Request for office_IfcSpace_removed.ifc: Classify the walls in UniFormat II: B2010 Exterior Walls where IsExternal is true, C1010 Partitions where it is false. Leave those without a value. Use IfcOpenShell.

First a look at what the model holds.

```python
import ifcopenshell
import ifcopenshell.util.element

model = ifcopenshell.open("office_IfcSpace_removed.ifc")
print(model.schema)
print("classifications:", [c.Name for c in model.by_type("IfcClassification")])
values = [ifcopenshell.util.element.get_pset(e, "Pset_WallCommon", "IsExternal") for e in model.by_type("IfcWall")]
for value in (True, False, None):
    print("IsExternal", value, values.count(value))
```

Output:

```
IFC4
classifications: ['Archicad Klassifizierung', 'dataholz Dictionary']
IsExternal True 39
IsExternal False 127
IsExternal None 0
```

```python
import ifcopenshell
import ifcopenshell.api.classification
import ifcopenshell.util.element

model = ifcopenshell.open("office_IfcSpace_removed.ifc")

system = ifcopenshell.api.classification.add_classification(model, classification="UniFormat II")

walls = model.by_type("IfcWall")
external = {e: ifcopenshell.util.element.get_pset(e, "Pset_WallCommon", "IsExternal") for e in walls}
for flag, code, name in ((True, "B2010", "Exterior Walls"), (False, "C1010", "Partitions")):
    products = [e for e in walls if external[e] is flag]
    ifcopenshell.api.classification.add_reference(
        model, products=products, classification=system, identification=code, name=name
    )
    print(code, len(products))

model.write("office_IfcSpace_removed_v2.ifc")
```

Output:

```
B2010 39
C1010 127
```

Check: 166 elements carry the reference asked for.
